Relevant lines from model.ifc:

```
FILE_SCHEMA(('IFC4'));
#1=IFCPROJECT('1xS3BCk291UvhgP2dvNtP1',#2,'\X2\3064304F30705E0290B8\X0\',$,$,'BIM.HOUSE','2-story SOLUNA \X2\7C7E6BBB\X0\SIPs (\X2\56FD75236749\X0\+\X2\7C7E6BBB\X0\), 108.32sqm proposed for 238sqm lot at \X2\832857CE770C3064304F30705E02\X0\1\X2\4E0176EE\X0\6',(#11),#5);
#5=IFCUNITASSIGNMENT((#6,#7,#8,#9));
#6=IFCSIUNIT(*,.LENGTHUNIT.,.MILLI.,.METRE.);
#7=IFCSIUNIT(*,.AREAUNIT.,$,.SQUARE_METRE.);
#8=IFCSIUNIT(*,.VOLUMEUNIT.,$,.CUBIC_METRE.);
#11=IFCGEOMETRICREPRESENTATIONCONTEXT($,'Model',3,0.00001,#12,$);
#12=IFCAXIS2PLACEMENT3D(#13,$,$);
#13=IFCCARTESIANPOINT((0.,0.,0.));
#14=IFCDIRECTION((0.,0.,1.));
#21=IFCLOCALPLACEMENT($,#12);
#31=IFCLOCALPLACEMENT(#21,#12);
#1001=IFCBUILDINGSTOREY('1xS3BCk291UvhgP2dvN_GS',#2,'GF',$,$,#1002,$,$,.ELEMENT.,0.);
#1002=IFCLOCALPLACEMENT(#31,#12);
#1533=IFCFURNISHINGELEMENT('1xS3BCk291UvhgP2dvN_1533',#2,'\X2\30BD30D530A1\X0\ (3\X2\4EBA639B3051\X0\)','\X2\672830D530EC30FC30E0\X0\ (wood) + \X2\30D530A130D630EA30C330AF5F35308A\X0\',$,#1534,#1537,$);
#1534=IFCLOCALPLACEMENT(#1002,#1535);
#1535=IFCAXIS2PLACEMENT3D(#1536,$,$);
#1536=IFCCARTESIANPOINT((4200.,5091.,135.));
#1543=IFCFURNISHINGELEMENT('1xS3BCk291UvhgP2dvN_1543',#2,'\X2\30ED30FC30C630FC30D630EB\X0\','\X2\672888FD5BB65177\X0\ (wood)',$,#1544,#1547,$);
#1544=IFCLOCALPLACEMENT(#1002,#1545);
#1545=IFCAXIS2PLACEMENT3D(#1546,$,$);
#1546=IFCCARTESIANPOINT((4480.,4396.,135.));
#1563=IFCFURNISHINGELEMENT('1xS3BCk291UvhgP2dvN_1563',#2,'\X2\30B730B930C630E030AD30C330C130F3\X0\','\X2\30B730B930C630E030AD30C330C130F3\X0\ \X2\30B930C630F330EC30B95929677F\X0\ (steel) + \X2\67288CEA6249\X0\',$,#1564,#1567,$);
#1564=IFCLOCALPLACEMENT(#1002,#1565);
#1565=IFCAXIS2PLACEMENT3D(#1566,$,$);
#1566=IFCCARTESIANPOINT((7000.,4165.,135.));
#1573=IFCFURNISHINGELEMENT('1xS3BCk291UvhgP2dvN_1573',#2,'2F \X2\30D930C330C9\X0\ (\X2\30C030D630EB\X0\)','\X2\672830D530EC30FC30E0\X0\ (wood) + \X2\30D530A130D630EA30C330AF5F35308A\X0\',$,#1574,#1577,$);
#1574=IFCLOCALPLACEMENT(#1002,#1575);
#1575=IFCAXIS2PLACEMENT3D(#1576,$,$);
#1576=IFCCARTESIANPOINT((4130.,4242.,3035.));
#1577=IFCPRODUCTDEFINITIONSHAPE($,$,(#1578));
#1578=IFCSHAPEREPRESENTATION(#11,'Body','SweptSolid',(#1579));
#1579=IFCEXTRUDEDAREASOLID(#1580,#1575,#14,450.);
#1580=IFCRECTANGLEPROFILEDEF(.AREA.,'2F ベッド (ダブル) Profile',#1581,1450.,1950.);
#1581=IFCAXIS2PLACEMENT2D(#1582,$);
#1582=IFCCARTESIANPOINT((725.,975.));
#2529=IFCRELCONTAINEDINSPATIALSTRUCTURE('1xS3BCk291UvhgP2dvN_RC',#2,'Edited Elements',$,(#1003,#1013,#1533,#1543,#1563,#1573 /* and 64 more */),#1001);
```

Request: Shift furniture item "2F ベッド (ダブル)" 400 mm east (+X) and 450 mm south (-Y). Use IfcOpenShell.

```python
import ifcopenshell
import ifcopenshell.api.geometry
import ifcopenshell.util.placement

model = ifcopenshell.open("model.ifc")

item = model.by_guid("1xS3BCk291UvhgP2dvN_1573")
matrix = ifcopenshell.util.placement.get_local_placement(item.ObjectPlacement)
matrix[0, 3] += 400.0
matrix[1, 3] -= 450.0
ifcopenshell.api.geometry.edit_object_placement(model, product=item, matrix=matrix, is_si=False)

print(ifcopenshell.util.placement.get_local_placement(item.ObjectPlacement).round(3) + 0.0)

model.write("model_v2.ifc")
```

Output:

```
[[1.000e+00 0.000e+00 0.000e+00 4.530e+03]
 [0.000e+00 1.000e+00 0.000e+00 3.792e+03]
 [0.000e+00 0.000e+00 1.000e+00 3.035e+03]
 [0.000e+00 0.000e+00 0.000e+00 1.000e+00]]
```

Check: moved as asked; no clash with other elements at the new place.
